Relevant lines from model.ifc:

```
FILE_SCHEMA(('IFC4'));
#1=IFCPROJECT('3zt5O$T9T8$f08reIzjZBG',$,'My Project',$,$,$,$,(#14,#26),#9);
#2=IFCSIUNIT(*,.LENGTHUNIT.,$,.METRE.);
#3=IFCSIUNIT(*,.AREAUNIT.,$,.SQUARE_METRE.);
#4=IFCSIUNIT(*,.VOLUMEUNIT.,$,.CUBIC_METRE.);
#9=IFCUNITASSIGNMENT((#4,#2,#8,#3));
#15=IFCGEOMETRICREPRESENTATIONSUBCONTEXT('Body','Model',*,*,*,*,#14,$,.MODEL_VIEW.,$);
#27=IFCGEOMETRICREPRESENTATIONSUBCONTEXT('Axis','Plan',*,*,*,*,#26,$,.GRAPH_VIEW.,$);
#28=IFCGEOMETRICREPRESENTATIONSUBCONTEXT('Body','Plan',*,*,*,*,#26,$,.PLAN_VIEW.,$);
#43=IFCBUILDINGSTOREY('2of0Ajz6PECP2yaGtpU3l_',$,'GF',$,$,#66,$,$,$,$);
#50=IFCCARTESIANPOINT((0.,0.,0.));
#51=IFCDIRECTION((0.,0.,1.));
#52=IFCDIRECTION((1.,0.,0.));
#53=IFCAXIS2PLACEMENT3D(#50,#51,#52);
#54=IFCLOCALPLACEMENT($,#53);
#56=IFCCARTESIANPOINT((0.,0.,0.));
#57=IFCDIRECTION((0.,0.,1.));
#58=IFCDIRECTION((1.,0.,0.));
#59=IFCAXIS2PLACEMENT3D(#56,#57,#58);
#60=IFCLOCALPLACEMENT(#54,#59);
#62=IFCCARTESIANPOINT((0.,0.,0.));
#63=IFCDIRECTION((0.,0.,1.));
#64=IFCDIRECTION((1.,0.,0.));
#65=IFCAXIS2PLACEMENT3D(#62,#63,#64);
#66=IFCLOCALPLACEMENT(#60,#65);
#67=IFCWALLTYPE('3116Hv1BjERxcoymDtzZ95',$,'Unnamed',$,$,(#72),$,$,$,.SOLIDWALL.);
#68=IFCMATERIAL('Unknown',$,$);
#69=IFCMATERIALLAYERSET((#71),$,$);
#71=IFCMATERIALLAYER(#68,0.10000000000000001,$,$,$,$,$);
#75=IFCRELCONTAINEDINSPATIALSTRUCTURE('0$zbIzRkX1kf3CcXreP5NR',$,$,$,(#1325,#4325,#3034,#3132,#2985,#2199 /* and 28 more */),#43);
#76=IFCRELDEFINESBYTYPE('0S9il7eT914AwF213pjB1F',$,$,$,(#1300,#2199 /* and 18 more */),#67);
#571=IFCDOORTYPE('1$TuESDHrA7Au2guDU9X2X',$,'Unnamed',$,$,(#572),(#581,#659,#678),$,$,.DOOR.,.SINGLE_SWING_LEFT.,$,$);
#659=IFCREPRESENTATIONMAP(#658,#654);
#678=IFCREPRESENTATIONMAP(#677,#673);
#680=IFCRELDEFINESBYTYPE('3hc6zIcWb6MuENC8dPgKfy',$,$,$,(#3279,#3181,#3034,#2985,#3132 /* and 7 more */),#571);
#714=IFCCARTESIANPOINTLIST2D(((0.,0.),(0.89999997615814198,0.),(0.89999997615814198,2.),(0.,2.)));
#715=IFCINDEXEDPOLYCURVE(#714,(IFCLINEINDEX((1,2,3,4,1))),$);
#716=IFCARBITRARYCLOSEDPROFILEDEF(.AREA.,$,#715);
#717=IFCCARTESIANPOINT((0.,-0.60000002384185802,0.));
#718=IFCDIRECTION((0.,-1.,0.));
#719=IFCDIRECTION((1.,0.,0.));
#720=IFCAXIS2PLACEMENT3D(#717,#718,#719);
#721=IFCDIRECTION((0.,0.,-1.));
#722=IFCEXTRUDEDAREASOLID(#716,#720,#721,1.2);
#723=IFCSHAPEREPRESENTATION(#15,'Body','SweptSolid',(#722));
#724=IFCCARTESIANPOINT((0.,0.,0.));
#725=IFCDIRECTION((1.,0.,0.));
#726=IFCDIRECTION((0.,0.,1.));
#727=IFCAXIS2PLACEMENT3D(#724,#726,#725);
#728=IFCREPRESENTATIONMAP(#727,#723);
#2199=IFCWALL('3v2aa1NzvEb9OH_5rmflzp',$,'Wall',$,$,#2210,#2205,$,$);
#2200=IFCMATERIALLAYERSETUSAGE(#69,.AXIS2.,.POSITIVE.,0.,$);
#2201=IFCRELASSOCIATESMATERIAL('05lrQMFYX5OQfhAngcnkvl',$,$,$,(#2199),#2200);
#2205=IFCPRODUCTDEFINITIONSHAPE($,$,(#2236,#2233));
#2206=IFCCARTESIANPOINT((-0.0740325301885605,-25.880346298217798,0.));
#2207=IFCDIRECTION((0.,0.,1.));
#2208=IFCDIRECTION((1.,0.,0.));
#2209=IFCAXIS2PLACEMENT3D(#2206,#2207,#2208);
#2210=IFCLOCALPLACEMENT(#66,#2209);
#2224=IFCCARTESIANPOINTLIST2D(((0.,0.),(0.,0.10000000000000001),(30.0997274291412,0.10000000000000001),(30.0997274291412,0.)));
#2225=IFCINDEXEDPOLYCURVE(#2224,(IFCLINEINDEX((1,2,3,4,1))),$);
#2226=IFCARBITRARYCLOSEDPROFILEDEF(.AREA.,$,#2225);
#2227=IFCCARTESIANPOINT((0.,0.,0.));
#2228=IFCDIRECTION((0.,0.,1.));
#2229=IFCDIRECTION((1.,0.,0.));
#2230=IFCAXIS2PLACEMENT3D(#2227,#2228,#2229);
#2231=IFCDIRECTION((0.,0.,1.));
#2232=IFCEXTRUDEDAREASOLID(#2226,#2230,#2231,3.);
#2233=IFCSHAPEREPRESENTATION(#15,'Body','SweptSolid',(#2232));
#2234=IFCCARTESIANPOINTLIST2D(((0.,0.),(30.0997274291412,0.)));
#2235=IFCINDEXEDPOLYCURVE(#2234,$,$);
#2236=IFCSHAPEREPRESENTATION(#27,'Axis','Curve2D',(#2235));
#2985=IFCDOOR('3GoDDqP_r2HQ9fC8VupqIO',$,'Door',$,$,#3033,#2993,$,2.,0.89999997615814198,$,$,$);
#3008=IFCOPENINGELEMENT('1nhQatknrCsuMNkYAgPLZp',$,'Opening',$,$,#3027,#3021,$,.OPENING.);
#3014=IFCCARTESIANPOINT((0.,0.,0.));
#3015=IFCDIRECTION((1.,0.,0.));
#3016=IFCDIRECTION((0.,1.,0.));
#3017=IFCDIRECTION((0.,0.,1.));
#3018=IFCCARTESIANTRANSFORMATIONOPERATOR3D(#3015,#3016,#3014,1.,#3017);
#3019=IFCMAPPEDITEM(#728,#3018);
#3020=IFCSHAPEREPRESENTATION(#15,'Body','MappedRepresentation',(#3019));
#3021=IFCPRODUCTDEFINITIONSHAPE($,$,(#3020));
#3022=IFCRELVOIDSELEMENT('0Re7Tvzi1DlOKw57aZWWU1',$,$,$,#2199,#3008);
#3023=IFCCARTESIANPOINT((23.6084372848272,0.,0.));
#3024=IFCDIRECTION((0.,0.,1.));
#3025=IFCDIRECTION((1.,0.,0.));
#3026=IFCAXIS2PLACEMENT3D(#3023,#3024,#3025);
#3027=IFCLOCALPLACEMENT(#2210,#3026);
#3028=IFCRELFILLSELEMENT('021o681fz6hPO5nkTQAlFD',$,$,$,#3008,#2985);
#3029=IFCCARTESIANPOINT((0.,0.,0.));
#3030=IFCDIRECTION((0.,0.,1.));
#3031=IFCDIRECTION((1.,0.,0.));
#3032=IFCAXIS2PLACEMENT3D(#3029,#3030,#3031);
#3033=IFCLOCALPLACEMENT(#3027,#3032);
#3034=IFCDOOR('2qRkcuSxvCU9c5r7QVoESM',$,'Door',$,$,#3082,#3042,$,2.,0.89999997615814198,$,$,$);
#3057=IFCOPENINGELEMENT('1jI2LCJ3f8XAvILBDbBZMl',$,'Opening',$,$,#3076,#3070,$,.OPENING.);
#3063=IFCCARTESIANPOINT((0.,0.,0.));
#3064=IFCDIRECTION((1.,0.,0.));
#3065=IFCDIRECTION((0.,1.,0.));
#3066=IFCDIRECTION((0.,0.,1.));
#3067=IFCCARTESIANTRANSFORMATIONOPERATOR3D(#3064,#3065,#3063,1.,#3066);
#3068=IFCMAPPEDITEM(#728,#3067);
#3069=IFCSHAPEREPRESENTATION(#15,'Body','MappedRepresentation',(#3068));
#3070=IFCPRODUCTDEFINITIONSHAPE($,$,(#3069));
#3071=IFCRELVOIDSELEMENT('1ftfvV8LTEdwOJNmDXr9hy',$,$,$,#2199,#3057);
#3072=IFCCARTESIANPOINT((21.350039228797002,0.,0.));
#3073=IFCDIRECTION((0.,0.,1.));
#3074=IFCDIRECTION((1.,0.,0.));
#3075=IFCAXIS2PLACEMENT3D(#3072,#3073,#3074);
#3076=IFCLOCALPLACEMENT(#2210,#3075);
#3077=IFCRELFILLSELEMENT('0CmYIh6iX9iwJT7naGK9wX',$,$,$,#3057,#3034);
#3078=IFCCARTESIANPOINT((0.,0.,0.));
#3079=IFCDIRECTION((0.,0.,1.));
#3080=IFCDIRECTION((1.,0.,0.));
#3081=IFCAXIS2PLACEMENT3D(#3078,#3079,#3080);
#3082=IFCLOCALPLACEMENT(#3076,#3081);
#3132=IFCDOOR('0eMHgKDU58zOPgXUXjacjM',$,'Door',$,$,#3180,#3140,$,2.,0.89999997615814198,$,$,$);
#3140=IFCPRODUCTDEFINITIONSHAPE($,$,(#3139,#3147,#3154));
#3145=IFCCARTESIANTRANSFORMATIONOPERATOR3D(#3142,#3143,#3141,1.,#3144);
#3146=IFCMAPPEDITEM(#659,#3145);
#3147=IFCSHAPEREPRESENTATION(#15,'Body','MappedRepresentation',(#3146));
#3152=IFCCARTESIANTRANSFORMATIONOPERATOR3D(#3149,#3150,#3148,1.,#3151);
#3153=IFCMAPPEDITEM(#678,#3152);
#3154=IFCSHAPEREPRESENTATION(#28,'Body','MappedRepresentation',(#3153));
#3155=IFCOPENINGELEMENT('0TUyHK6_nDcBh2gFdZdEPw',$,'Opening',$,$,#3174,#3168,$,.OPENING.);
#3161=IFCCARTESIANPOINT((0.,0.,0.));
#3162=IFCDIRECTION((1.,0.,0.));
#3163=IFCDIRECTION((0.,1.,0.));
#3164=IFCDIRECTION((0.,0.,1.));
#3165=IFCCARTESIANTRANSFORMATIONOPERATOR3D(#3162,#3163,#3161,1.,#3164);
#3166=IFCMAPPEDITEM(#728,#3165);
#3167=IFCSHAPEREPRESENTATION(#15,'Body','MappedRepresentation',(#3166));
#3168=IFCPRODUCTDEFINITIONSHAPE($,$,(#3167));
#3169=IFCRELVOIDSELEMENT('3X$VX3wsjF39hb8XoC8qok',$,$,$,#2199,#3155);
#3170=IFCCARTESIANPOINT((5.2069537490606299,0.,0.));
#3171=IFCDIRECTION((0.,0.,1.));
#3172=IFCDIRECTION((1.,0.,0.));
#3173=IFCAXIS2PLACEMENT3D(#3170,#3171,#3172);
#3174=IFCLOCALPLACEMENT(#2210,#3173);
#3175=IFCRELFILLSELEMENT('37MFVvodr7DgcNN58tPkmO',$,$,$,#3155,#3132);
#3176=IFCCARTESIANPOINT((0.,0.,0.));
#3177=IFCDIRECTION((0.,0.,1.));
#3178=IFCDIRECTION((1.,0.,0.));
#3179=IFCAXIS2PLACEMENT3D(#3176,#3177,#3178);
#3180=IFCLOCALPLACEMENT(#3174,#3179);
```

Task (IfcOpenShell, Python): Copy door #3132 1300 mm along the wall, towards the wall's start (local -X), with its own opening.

```python
import ifcopenshell
import ifcopenshell.api.feature
import ifcopenshell.api.geometry
import ifcopenshell.api.root
import ifcopenshell.geom
import ifcopenshell.util.element
import ifcopenshell.util.placement
import ifcopenshell.util.shape
import ifcopenshell.util.unit

model = ifcopenshell.open("model.ifc")
unit_scale = ifcopenshell.util.unit.calculate_unit_scale(model)
settings = ifcopenshell.geom.settings()


def volume(element):
    """Net volume in cubic metres, openings subtracted."""
    shape = ifcopenshell.geom.create_shape(settings, element)
    return ifcopenshell.util.shape.get_volume(shape.geometry)


door = model.by_guid("0eMHgKDU58zOPgXUXjacjM")
opening = door.FillsVoids[0].RelatingOpeningElement
wall = opening.VoidsElements[0].RelatingBuildingElement
before = volume(wall)
shift = ifcopenshell.util.placement.get_local_placement(wall.ObjectPlacement)[:3, 0] * -1.3 / unit_scale

# copy_class copies the void relationship, type, container and properties, but no geometry.
new_opening = ifcopenshell.api.root.copy_class(model, product=opening)
new_opening.Representation = ifcopenshell.util.element.copy_deep(
    model, opening.Representation, exclude=["IfcGeometricRepresentationContext", "IfcRepresentationMap"]
)
new_door = ifcopenshell.api.root.copy_class(model, product=door)
new_door.Representation = ifcopenshell.util.element.copy_deep(
    model, door.Representation, exclude=["IfcGeometricRepresentationContext", "IfcRepresentationMap"]
)
ifcopenshell.api.feature.add_filling(model, opening=new_opening, element=new_door)

for old, new in ((opening, new_opening), (door, new_door)):
    matrix = ifcopenshell.util.placement.get_local_placement(old.ObjectPlacement)
    matrix[:3, 3] += shift
    ifcopenshell.api.geometry.edit_object_placement(model, product=new, matrix=matrix, is_si=False)

after = volume(wall)

print(f"wall volume {before:.3f} -> {after:.3f} m3")

model.write("model_v2.ifc")
```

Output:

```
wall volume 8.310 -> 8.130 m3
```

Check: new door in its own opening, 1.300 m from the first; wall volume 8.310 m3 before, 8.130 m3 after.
